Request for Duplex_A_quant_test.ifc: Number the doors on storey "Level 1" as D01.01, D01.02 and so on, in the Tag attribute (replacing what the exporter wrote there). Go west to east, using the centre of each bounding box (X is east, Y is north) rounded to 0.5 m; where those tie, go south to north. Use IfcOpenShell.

First a look at what the model holds.

```python
import ifcopenshell
import ifcopenshell.util.element
import ifcopenshell.util.placement

model = ifcopenshell.open("Duplex_A_quant_test.ifc")
print(model.schema)
storey = next(s for s in model.by_type("IfcBuildingStorey") if s.Name == "Level 1")
doors = [e for e in ifcopenshell.util.element.get_decomposition(storey) if e.is_a("IfcDoor")]
for e in sorted(doors, key=lambda e: e.id()):
    origin = ifcopenshell.util.placement.get_local_placement(e.ObjectPlacement)[:3, 3]
    print(e.id(), e.Tag, e.Name, origin.round(2) + 0.0, sep=" | ")
```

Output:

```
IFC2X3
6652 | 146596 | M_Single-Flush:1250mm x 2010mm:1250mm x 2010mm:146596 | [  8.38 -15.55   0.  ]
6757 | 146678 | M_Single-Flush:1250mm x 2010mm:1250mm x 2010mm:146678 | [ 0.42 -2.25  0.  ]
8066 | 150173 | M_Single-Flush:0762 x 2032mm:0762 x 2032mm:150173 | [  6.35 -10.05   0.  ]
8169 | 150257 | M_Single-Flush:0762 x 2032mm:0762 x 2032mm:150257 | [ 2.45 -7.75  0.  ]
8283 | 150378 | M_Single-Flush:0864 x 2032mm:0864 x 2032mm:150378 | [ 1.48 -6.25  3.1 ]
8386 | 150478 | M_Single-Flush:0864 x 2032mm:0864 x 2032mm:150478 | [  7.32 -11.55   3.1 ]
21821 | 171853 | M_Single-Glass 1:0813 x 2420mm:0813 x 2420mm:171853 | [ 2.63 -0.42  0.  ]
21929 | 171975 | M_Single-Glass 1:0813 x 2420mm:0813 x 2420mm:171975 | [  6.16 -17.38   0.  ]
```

```python
import ifcopenshell
import ifcopenshell.geom
import ifcopenshell.util.element
import ifcopenshell.util.shape

model = ifcopenshell.open("Duplex_A_quant_test.ifc")
settings = ifcopenshell.geom.settings()
settings.set("use-world-coords", True)


def centre(element):
    shape = ifcopenshell.geom.create_shape(settings, element)
    return ifcopenshell.util.shape.get_bbox_centroid(shape.geometry)


storey = next(s for s in model.by_type("IfcBuildingStorey") if s.Name == "Level 1")
doors = [e for e in ifcopenshell.util.element.get_decomposition(storey) if e.is_a("IfcDoor")]

# Insertion points can sit at a corner or the storey origin, so sort by the geometry (in metres).
centres = {e: centre(e) for e in doors}
doors.sort(key=lambda e: (round(centres[e][0] / 0.5), centres[e][1]))

for i, e in enumerate(doors, start=1):
    number = f"D01.{i:02d}"
    e.Tag = number
    print(e.id(), number)

model.write("Duplex_A_quant_test_edited.ifc")
```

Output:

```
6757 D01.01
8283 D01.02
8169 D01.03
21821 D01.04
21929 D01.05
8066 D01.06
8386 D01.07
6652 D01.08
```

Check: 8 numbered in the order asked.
